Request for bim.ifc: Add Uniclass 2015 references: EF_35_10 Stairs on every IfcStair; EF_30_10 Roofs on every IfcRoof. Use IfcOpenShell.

First a look at what the model holds.

```python
import ifcopenshell

model = ifcopenshell.open("bim.ifc")
print(model.schema)
print("classifications:", [c.Name for c in model.by_type("IfcClassification")])
for ifc_class in ("IfcDoor", "IfcRoof", "IfcStair", "IfcWall", "IfcWindow"):
    print(ifc_class, len(model.by_type(ifc_class)))
```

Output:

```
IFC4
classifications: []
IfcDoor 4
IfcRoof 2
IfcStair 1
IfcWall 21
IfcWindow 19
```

```python
import ifcopenshell
import ifcopenshell.api.classification

model = ifcopenshell.open("bim.ifc")

system = ifcopenshell.api.classification.add_classification(model, classification="Uniclass 2015")

codes = {
    "IfcStair": ("EF_35_10", "Stairs"),
    "IfcRoof": ("EF_30_10", "Roofs"),
}
for ifc_class, (code, name) in codes.items():
    products = model.by_type(ifc_class)
    ifcopenshell.api.classification.add_reference(
        model, products=products, classification=system, identification=code, name=name
    )
    print(code, len(products))

model.write("bim_updated.ifc")
```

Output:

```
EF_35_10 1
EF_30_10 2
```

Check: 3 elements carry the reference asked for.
